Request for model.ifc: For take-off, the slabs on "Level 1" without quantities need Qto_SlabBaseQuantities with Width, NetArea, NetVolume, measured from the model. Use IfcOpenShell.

First a look at what the model holds.

```python
import ifcopenshell
import ifcopenshell.util.element
import ifcopenshell.util.unit

model = ifcopenshell.open("model.ifc")
print(model.schema)
for unit_type in ("LENGTHUNIT", "AREAUNIT", "VOLUMEUNIT"):
    print(unit_type, ifcopenshell.util.unit.calculate_unit_scale(model, unit_type))
storey = next(s for s in model.by_type("IfcBuildingStorey") if s.Name == "Level 1")
slabs = [e for e in ifcopenshell.util.element.get_decomposition(storey) if e.is_a("IfcSlab")]
for e in sorted(slabs, key=lambda e: e.id()):
    print(e.id(), e.is_a(), e.Name, list(ifcopenshell.util.element.get_psets(e, qtos_only=True)), sep=" | ")
```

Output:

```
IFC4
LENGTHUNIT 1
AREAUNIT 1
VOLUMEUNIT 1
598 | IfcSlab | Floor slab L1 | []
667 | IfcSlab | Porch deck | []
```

```python
import ifcopenshell
import ifcopenshell.api.pset
import ifcopenshell.geom
import ifcopenshell.util.element
import ifcopenshell.util.shape
import ifcopenshell.util.unit

model = ifcopenshell.open("model.ifc")
unit_scale = ifcopenshell.util.unit.calculate_unit_scale(model)
area_scale = ifcopenshell.util.unit.calculate_unit_scale(model, "AREAUNIT")
volume_scale = ifcopenshell.util.unit.calculate_unit_scale(model, "VOLUMEUNIT")
settings = ifcopenshell.geom.settings()

storey = next(s for s in model.by_type("IfcBuildingStorey") if s.Name == "Level 1")
slabs = [e for e in ifcopenshell.util.element.get_decomposition(storey) if e.is_a("IfcSlab")]

for e in sorted(slabs, key=lambda e: e.id()):
    if ifcopenshell.util.element.get_psets(e, qtos_only=True, should_inherit=False):
        continue
    # Geometry comes back in metres, in the element's own axes.
    shape = ifcopenshell.geom.create_shape(settings, e)
    values = {
        "Width": ifcopenshell.util.shape.get_z(shape.geometry) / unit_scale,
        "NetArea": ifcopenshell.util.shape.get_footprint_area(shape.geometry) / area_scale,
        "NetVolume": ifcopenshell.util.shape.get_volume(shape.geometry) / volume_scale,
    }
    qto = ifcopenshell.api.pset.add_qto(model, product=e, name="Qto_SlabBaseQuantities")
    ifcopenshell.api.pset.edit_qto(model, qto=qto, properties=values)
    print(e.id(), {k: round(v, 3) for k, v in values.items()})

model.write("model_rev.ifc")
```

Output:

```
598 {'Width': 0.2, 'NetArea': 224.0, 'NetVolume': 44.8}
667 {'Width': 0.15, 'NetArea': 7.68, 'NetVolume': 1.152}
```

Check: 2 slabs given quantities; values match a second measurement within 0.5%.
